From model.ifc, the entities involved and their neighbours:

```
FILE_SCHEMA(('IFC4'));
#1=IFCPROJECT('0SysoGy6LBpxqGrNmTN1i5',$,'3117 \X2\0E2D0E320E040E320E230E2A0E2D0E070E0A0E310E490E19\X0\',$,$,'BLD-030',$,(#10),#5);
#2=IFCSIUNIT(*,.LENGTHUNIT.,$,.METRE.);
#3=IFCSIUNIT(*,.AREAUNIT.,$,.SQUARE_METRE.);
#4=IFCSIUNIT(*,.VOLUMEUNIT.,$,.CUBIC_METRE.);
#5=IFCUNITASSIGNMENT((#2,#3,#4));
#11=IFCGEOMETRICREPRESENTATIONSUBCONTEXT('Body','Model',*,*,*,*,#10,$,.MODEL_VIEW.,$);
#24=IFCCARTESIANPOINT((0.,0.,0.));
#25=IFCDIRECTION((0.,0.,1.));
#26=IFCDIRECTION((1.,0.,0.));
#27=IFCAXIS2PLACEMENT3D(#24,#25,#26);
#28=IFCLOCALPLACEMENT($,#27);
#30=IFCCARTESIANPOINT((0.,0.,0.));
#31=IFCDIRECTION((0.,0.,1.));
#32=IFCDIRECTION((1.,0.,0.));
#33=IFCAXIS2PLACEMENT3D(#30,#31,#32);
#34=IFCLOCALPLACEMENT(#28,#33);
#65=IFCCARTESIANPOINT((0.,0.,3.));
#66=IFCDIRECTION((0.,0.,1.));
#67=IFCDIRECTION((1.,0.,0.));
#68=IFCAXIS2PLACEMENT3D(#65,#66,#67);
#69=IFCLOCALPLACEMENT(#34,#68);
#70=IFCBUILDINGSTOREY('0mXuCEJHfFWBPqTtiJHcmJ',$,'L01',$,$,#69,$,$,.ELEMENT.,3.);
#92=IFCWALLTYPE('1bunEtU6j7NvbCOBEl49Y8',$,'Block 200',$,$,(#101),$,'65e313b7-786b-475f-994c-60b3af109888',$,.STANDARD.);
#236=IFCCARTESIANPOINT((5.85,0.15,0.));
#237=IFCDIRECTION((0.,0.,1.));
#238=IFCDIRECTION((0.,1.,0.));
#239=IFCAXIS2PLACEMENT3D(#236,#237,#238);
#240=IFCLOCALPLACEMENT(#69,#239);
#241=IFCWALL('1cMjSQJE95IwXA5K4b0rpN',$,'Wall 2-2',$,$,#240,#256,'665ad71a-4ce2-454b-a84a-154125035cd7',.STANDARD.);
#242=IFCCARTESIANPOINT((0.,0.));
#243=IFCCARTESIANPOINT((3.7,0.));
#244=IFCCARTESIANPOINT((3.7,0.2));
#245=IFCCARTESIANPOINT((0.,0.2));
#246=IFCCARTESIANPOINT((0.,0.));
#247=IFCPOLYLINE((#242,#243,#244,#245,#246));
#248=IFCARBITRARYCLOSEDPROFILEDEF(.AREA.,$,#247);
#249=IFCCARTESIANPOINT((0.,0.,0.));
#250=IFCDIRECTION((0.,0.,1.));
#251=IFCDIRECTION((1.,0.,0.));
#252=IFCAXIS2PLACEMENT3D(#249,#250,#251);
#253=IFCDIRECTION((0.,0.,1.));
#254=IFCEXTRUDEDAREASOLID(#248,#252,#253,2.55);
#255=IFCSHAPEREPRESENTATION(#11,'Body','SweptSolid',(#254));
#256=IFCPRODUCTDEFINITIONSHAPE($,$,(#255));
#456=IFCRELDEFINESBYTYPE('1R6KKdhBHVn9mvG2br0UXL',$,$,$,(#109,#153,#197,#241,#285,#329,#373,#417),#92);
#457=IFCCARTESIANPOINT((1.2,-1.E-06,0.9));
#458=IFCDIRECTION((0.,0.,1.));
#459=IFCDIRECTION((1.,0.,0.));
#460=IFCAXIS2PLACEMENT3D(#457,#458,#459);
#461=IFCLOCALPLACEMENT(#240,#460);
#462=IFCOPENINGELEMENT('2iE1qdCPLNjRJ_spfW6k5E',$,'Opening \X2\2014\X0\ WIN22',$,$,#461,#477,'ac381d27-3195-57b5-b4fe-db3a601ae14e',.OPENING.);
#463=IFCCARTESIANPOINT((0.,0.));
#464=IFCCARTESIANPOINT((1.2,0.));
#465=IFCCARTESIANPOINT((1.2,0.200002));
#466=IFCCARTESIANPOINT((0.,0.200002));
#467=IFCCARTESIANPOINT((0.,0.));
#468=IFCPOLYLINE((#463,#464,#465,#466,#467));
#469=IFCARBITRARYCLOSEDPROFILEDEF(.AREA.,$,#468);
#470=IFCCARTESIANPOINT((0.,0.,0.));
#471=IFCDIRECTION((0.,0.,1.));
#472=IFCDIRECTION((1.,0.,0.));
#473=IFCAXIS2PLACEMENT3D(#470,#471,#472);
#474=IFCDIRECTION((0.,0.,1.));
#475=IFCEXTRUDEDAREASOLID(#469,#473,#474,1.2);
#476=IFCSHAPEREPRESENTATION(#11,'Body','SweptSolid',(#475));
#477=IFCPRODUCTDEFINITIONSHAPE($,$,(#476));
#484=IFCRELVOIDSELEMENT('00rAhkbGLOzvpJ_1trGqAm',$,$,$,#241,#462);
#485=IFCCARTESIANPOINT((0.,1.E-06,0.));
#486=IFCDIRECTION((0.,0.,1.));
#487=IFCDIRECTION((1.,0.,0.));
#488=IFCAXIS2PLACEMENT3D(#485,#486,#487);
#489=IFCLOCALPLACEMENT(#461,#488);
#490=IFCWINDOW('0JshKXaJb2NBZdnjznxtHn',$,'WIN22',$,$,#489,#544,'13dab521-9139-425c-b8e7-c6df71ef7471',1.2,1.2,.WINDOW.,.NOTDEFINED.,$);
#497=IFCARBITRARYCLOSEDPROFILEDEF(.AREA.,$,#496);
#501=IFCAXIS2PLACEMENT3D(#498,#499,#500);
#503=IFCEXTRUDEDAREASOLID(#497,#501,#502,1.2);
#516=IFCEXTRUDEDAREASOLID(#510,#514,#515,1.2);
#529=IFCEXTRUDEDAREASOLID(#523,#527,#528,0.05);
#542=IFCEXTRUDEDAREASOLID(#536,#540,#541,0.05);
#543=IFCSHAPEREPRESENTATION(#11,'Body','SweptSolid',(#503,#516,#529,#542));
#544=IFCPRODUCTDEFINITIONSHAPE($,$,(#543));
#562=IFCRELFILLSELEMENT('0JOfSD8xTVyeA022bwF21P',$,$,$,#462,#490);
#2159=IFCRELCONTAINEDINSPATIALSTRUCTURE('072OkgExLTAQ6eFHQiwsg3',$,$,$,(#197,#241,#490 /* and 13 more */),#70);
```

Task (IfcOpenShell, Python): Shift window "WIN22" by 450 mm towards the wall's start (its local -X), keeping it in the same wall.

```python
import ifcopenshell
import ifcopenshell.api.geometry
import ifcopenshell.util.placement

model = ifcopenshell.open("model.ifc")

window = model.by_id(490)
opening = window.FillsVoids[0].RelatingOpeningElement
wall = opening.VoidsElements[0].RelatingBuildingElement

wall_matrix = ifcopenshell.util.placement.get_local_placement(wall.ObjectPlacement)
shift = wall_matrix[:3, 0] * -0.45
before = ifcopenshell.util.placement.get_local_placement(window.ObjectPlacement)[:3, 3].copy()

# The window is placed relative to its opening, so it follows when the opening moves.
matrix = ifcopenshell.util.placement.get_local_placement(opening.ObjectPlacement)
matrix[:3, 3] += shift
ifcopenshell.api.geometry.edit_object_placement(
    model, product=opening, matrix=matrix, is_si=False, should_transform_children=True
)

after = ifcopenshell.util.placement.get_local_placement(window.ObjectPlacement)[:3, 3]
print("window moved by", (after - before).round(3) + 0.0)

model.write("model-out.ifc")
```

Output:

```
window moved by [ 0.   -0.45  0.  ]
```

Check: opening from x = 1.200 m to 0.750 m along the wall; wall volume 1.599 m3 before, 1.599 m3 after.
